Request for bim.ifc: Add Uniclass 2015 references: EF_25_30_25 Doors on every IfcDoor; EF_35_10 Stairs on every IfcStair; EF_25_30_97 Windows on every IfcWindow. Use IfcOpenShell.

First a look at what the model holds.

```python
import ifcopenshell

model = ifcopenshell.open("bim.ifc")
print(model.schema)
print("classifications:", [c.Name for c in model.by_type("IfcClassification")])
for ifc_class in ("IfcDoor", "IfcRoof", "IfcStair", "IfcWall", "IfcWindow"):
    print(ifc_class, len(model.by_type(ifc_class)))
```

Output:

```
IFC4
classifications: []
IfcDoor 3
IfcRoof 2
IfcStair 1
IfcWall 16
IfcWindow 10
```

```python
import ifcopenshell
import ifcopenshell.api.classification

model = ifcopenshell.open("bim.ifc")

system = ifcopenshell.api.classification.add_classification(model, classification="Uniclass 2015")

codes = {
    "IfcDoor": ("EF_25_30_25", "Doors"),
    "IfcStair": ("EF_35_10", "Stairs"),
    "IfcWindow": ("EF_25_30_97", "Windows"),
}
for ifc_class, (code, name) in codes.items():
    products = model.by_type(ifc_class)
    ifcopenshell.api.classification.add_reference(
        model, products=products, classification=system, identification=code, name=name
    )
    print(code, len(products))

model.write("bim_updated.ifc")
```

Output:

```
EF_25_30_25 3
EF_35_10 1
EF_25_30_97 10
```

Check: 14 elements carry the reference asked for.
